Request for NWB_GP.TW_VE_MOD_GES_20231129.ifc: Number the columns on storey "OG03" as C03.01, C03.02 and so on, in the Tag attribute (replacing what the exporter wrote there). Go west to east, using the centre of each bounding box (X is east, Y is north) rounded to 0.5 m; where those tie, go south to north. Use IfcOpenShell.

First a look at what the model holds.

```python
import ifcopenshell
import ifcopenshell.util.element
import ifcopenshell.util.placement

model = ifcopenshell.open("NWB_GP.TW_VE_MOD_GES_20231129.ifc")
print(model.schema)
storey = next(s for s in model.by_type("IfcBuildingStorey") if s.Name == "OG03")
columns = [e for e in ifcopenshell.util.element.get_decomposition(storey) if e.is_a("IfcColumn")]
for e in sorted(columns, key=lambda e: e.id()):
    origin = ifcopenshell.util.placement.get_local_placement(e.ObjectPlacement)[:3, 3]
    print(e.id(), e.Tag, e.Name, origin.round(2) + 0.0, sep=" | ")
```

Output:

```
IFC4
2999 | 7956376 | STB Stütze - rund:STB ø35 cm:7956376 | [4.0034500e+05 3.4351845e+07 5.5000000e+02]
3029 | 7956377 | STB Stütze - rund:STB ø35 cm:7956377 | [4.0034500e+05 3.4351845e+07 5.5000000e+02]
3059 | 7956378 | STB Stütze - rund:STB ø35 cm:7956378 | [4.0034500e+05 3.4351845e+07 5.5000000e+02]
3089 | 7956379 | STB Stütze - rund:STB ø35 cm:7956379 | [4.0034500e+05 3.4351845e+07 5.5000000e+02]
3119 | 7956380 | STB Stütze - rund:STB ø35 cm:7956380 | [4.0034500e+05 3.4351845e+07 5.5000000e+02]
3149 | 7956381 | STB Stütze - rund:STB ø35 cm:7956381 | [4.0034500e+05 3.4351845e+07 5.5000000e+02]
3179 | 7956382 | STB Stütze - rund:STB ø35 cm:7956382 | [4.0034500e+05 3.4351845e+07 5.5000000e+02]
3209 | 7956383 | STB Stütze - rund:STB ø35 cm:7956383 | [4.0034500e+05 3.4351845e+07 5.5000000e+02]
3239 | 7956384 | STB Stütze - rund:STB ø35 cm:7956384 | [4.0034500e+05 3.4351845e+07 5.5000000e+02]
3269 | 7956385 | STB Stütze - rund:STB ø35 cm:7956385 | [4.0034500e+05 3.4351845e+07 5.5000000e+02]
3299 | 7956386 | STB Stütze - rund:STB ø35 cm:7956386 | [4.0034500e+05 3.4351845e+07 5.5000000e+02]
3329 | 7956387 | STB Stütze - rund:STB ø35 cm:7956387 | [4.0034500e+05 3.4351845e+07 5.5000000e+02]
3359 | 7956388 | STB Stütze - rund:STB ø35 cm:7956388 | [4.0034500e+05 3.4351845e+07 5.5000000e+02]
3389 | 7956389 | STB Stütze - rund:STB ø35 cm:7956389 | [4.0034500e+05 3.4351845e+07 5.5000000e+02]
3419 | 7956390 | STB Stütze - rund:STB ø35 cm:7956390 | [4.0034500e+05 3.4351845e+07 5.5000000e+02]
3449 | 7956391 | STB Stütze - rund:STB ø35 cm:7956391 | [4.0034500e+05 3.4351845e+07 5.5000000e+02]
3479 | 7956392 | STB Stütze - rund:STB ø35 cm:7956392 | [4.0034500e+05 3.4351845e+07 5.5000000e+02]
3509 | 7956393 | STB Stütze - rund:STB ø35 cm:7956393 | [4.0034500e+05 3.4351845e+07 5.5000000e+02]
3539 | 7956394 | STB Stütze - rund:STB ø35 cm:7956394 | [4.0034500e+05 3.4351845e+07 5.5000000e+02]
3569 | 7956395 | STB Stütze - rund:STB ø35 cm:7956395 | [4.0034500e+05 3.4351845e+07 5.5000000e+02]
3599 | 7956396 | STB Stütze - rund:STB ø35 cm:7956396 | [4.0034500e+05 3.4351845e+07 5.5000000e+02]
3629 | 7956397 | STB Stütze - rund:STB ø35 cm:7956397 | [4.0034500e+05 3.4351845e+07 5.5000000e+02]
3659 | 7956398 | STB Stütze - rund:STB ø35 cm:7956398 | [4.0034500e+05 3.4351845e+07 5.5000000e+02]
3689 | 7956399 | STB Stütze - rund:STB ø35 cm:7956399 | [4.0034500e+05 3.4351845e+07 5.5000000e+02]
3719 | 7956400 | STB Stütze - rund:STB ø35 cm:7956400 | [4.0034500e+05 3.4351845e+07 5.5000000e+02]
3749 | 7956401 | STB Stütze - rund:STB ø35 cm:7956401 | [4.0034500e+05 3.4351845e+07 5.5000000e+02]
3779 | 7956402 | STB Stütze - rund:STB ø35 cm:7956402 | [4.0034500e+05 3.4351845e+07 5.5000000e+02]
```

```python
import ifcopenshell
import ifcopenshell.geom
import ifcopenshell.util.element
import ifcopenshell.util.shape

model = ifcopenshell.open("NWB_GP.TW_VE_MOD_GES_20231129.ifc")
settings = ifcopenshell.geom.settings()
settings.set("use-world-coords", True)


def centre(element):
    shape = ifcopenshell.geom.create_shape(settings, element)
    return ifcopenshell.util.shape.get_bbox_centroid(shape.geometry)


storey = next(s for s in model.by_type("IfcBuildingStorey") if s.Name == "OG03")
columns = [e for e in ifcopenshell.util.element.get_decomposition(storey) if e.is_a("IfcColumn")]

# Insertion points can sit at a corner or the storey origin, so sort by the geometry (in metres).
centres = {e: centre(e) for e in columns}
columns.sort(key=lambda e: (round(centres[e][0] / 0.5), centres[e][1]))

for i, e in enumerate(columns, start=1):
    number = f"C03.{i:02d}"
    e.Tag = number
    print(e.id(), number)

model.write("NWB_GP.TW_VE_MOD_GES_20231129-out.ifc")
```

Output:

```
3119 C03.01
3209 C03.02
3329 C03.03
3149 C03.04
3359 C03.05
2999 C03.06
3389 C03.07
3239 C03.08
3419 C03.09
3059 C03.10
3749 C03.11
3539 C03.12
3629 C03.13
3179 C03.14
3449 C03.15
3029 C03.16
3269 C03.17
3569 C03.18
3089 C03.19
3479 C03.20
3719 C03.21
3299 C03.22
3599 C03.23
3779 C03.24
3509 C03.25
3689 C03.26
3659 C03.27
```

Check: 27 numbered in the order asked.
